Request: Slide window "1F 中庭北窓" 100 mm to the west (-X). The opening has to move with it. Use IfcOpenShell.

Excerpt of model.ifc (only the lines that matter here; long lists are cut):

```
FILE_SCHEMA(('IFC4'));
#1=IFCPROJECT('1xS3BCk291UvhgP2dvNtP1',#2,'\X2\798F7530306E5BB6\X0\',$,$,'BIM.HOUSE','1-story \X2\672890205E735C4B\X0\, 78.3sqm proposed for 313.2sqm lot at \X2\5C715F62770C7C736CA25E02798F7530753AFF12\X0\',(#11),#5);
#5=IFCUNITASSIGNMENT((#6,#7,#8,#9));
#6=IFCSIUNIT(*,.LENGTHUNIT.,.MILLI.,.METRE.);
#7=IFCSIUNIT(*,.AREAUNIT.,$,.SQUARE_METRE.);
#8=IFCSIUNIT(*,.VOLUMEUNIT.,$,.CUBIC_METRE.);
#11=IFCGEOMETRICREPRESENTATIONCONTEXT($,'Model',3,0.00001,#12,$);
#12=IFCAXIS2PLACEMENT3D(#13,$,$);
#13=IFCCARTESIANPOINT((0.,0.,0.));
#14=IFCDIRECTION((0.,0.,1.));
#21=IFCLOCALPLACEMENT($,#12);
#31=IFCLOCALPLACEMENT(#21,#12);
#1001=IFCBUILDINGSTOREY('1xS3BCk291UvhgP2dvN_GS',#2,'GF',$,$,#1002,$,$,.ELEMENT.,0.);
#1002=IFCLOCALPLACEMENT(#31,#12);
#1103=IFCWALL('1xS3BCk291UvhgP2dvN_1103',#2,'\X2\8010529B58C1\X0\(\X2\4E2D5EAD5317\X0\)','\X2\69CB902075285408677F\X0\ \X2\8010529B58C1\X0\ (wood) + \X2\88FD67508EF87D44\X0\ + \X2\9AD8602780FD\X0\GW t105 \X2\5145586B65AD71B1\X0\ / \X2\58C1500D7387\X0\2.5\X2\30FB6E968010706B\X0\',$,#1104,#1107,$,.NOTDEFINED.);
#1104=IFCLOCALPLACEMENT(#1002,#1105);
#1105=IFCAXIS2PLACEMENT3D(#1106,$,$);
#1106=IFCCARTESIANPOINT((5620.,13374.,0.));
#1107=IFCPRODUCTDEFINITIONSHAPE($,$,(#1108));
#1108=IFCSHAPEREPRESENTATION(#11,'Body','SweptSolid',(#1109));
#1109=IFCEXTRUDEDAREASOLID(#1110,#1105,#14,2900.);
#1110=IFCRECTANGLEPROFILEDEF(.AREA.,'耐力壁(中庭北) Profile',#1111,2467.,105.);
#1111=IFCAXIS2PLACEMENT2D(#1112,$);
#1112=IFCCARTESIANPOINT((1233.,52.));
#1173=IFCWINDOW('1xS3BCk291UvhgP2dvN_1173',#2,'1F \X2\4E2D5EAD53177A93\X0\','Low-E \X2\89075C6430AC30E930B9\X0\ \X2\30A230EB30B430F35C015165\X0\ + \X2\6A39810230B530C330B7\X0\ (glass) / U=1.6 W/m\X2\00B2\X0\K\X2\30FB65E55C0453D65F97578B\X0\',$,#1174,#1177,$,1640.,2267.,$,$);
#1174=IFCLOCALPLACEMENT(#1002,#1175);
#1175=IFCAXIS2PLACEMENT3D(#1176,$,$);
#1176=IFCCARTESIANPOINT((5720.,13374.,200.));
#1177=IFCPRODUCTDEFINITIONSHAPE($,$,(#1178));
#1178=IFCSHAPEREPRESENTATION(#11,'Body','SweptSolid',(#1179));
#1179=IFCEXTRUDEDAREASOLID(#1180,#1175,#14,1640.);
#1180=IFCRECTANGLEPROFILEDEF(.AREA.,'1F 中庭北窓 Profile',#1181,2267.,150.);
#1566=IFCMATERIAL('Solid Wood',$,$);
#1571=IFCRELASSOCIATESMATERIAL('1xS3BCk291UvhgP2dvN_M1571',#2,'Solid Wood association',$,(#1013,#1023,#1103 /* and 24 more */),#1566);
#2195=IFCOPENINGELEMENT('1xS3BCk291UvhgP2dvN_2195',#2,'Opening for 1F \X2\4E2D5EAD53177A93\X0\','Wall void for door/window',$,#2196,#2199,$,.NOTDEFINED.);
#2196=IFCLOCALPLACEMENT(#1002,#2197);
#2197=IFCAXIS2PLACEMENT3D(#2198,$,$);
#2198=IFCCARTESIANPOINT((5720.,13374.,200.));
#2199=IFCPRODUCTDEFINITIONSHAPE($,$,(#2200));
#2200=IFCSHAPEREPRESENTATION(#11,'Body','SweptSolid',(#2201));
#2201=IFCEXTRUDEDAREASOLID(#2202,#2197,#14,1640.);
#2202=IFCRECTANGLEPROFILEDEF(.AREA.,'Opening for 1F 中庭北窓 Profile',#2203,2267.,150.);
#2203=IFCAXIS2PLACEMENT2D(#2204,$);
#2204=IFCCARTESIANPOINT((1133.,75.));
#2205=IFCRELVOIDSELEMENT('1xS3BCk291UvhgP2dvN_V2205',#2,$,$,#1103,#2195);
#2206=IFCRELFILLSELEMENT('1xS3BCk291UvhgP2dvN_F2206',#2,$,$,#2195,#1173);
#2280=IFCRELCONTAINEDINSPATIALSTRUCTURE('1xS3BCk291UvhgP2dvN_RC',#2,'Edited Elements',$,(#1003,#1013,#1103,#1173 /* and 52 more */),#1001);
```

```python
import ifcopenshell
import ifcopenshell.api.geometry
import ifcopenshell.util.placement

model = ifcopenshell.open("model.ifc")

window = model.by_guid("1xS3BCk291UvhgP2dvN_1173")
opening = window.FillsVoids[0].RelatingOpeningElement
wall = opening.VoidsElements[0].RelatingBuildingElement

wall_matrix = ifcopenshell.util.placement.get_local_placement(wall.ObjectPlacement)
shift = wall_matrix[:3, 0] * -100.0
before = ifcopenshell.util.placement.get_local_placement(window.ObjectPlacement)[:3, 3].copy()

# The window is not placed relative to its opening, so move both.
for product in (opening, window):
    matrix = ifcopenshell.util.placement.get_local_placement(product.ObjectPlacement)
    matrix[:3, 3] += shift
    ifcopenshell.api.geometry.edit_object_placement(model, product=product, matrix=matrix, is_si=False)

after = ifcopenshell.util.placement.get_local_placement(window.ObjectPlacement)[:3, 3]
print("window moved by", (after - before).round(3) + 0.0)

model.write("model_rev.ifc")
```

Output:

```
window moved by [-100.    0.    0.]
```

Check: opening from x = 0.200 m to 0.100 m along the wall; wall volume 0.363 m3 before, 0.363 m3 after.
